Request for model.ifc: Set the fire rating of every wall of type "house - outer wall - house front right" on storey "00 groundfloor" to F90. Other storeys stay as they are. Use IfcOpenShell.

First a look at what the model holds.

```python
import ifcopenshell
import ifcopenshell.util.element

model = ifcopenshell.open("model.ifc")
print(model.schema)
storey = next(s for s in model.by_type("IfcBuildingStorey") if s.Name == "00 groundfloor")
walls = [e for e in ifcopenshell.util.element.get_decomposition(storey) if e.is_a("IfcWall")]
seen = {}
for e in walls:
    element_type = ifcopenshell.util.element.get_type(e)
    key = (element_type.Name if element_type != e and element_type else None, ifcopenshell.util.element.get_pset(e, "Pset_WallCommon", "FireRating"))
    seen[key] = seen.get(key, 0) + 1
for (name, value), count in sorted(seen.items(), key=str):
    print(count, "x", name, "|", value)
```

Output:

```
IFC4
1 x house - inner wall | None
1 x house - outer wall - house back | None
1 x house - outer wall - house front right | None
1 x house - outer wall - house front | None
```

```python
import ifcopenshell
import ifcopenshell.api.pset
import ifcopenshell.util.element

model = ifcopenshell.open("model.ifc")

storey = next(s for s in model.by_type("IfcBuildingStorey") if s.Name == "00 groundfloor")
walls = [e for e in ifcopenshell.util.element.get_decomposition(storey) if e.is_a("IfcWall")]

count = 0
for e in walls:
    element_type = ifcopenshell.util.element.get_type(e)
    if element_type in (None, e) or element_type.Name != "house - outer wall - house front right":
        continue
    # add_pset returns the element's existing set when there is one.
    pset = ifcopenshell.api.pset.add_pset(model, product=e, name="Pset_WallCommon")
    ifcopenshell.api.pset.edit_pset(model, pset=pset, properties={"FireRating": "F90"})
    count += 1

print(count, "walls updated")

model.write("model-out.ifc")
```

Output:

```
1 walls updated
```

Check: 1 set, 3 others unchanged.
